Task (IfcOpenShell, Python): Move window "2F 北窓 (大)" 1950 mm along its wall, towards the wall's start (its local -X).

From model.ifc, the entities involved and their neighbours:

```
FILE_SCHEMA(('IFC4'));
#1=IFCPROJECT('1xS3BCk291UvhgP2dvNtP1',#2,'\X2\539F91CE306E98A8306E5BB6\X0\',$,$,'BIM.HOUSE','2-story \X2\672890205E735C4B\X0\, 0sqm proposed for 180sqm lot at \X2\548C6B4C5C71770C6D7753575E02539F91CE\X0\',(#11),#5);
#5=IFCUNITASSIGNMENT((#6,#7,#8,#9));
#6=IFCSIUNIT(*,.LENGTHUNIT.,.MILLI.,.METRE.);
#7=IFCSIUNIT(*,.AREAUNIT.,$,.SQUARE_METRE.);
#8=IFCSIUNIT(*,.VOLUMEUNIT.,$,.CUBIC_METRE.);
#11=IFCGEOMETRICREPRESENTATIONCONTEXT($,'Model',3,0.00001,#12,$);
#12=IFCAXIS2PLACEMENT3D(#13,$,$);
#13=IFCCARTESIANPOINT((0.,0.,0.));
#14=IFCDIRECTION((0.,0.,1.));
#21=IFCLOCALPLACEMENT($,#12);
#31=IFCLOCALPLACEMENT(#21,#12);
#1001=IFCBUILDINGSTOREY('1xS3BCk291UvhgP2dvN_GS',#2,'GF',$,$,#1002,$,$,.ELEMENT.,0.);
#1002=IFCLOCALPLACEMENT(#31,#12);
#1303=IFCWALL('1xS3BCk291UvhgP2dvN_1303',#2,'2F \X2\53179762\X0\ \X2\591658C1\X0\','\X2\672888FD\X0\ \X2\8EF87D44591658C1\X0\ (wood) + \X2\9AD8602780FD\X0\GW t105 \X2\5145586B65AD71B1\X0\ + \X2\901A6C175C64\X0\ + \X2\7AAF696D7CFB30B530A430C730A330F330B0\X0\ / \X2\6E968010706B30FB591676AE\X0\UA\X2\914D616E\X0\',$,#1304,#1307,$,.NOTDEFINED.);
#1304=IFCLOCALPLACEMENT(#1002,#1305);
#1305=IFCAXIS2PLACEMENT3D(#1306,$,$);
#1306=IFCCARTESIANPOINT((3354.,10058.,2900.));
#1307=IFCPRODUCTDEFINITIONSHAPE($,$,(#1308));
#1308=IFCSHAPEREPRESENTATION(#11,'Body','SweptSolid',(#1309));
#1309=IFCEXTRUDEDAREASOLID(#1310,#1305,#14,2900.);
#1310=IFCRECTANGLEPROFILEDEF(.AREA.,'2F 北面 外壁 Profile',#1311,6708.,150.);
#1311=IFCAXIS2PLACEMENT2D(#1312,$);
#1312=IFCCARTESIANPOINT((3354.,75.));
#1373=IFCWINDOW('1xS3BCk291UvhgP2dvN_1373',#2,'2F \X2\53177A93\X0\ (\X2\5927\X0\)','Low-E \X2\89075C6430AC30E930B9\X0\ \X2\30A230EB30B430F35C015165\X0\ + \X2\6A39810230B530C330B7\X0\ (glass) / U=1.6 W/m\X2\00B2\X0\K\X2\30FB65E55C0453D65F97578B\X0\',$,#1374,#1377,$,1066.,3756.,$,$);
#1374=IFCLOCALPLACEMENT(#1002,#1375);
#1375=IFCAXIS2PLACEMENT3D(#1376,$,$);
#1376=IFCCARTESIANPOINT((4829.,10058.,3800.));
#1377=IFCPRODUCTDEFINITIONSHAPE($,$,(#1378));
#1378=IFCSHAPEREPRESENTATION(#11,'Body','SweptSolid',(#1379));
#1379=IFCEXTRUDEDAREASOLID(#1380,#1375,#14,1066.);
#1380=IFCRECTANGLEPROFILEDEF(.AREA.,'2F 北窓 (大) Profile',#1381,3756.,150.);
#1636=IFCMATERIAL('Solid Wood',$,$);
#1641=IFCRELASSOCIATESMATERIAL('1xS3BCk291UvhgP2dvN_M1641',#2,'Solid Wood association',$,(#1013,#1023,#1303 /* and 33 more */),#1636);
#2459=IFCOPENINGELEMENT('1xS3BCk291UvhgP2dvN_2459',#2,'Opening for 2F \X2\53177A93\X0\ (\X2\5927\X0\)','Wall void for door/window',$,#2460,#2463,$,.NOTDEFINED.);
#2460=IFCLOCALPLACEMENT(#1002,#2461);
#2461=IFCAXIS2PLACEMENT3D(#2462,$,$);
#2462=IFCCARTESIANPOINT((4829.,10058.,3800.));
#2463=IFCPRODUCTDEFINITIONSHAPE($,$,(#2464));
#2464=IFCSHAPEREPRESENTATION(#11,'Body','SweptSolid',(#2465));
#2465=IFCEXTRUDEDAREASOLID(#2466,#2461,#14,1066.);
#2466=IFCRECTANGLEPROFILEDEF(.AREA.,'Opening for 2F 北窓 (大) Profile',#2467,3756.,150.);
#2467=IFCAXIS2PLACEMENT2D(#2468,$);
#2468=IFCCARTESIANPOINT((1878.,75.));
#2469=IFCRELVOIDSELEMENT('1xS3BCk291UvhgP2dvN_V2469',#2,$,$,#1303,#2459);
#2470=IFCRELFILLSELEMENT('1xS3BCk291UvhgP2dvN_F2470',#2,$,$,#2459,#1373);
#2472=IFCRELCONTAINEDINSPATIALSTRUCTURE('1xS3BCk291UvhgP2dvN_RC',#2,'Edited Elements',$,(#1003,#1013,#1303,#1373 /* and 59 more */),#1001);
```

```python
import ifcopenshell
import ifcopenshell.api.geometry
import ifcopenshell.util.placement

model = ifcopenshell.open("model.ifc")

window = model.by_id(1373)
opening = window.FillsVoids[0].RelatingOpeningElement
wall = opening.VoidsElements[0].RelatingBuildingElement

wall_matrix = ifcopenshell.util.placement.get_local_placement(wall.ObjectPlacement)
shift = wall_matrix[:3, 0] * -1950.0
before = ifcopenshell.util.placement.get_local_placement(window.ObjectPlacement)[:3, 3].copy()

# The window is not placed relative to its opening, so move both.
for product in (opening, window):
    matrix = ifcopenshell.util.placement.get_local_placement(product.ObjectPlacement)
    matrix[:3, 3] += shift
    ifcopenshell.api.geometry.edit_object_placement(model, product=product, matrix=matrix, is_si=False)

after = ifcopenshell.util.placement.get_local_placement(window.ObjectPlacement)[:3, 3]
print("window moved by", (after - before).round(3) + 0.0)

model.write("model_edited.ifc")
```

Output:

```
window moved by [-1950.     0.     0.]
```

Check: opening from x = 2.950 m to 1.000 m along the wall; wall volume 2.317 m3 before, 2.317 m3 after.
